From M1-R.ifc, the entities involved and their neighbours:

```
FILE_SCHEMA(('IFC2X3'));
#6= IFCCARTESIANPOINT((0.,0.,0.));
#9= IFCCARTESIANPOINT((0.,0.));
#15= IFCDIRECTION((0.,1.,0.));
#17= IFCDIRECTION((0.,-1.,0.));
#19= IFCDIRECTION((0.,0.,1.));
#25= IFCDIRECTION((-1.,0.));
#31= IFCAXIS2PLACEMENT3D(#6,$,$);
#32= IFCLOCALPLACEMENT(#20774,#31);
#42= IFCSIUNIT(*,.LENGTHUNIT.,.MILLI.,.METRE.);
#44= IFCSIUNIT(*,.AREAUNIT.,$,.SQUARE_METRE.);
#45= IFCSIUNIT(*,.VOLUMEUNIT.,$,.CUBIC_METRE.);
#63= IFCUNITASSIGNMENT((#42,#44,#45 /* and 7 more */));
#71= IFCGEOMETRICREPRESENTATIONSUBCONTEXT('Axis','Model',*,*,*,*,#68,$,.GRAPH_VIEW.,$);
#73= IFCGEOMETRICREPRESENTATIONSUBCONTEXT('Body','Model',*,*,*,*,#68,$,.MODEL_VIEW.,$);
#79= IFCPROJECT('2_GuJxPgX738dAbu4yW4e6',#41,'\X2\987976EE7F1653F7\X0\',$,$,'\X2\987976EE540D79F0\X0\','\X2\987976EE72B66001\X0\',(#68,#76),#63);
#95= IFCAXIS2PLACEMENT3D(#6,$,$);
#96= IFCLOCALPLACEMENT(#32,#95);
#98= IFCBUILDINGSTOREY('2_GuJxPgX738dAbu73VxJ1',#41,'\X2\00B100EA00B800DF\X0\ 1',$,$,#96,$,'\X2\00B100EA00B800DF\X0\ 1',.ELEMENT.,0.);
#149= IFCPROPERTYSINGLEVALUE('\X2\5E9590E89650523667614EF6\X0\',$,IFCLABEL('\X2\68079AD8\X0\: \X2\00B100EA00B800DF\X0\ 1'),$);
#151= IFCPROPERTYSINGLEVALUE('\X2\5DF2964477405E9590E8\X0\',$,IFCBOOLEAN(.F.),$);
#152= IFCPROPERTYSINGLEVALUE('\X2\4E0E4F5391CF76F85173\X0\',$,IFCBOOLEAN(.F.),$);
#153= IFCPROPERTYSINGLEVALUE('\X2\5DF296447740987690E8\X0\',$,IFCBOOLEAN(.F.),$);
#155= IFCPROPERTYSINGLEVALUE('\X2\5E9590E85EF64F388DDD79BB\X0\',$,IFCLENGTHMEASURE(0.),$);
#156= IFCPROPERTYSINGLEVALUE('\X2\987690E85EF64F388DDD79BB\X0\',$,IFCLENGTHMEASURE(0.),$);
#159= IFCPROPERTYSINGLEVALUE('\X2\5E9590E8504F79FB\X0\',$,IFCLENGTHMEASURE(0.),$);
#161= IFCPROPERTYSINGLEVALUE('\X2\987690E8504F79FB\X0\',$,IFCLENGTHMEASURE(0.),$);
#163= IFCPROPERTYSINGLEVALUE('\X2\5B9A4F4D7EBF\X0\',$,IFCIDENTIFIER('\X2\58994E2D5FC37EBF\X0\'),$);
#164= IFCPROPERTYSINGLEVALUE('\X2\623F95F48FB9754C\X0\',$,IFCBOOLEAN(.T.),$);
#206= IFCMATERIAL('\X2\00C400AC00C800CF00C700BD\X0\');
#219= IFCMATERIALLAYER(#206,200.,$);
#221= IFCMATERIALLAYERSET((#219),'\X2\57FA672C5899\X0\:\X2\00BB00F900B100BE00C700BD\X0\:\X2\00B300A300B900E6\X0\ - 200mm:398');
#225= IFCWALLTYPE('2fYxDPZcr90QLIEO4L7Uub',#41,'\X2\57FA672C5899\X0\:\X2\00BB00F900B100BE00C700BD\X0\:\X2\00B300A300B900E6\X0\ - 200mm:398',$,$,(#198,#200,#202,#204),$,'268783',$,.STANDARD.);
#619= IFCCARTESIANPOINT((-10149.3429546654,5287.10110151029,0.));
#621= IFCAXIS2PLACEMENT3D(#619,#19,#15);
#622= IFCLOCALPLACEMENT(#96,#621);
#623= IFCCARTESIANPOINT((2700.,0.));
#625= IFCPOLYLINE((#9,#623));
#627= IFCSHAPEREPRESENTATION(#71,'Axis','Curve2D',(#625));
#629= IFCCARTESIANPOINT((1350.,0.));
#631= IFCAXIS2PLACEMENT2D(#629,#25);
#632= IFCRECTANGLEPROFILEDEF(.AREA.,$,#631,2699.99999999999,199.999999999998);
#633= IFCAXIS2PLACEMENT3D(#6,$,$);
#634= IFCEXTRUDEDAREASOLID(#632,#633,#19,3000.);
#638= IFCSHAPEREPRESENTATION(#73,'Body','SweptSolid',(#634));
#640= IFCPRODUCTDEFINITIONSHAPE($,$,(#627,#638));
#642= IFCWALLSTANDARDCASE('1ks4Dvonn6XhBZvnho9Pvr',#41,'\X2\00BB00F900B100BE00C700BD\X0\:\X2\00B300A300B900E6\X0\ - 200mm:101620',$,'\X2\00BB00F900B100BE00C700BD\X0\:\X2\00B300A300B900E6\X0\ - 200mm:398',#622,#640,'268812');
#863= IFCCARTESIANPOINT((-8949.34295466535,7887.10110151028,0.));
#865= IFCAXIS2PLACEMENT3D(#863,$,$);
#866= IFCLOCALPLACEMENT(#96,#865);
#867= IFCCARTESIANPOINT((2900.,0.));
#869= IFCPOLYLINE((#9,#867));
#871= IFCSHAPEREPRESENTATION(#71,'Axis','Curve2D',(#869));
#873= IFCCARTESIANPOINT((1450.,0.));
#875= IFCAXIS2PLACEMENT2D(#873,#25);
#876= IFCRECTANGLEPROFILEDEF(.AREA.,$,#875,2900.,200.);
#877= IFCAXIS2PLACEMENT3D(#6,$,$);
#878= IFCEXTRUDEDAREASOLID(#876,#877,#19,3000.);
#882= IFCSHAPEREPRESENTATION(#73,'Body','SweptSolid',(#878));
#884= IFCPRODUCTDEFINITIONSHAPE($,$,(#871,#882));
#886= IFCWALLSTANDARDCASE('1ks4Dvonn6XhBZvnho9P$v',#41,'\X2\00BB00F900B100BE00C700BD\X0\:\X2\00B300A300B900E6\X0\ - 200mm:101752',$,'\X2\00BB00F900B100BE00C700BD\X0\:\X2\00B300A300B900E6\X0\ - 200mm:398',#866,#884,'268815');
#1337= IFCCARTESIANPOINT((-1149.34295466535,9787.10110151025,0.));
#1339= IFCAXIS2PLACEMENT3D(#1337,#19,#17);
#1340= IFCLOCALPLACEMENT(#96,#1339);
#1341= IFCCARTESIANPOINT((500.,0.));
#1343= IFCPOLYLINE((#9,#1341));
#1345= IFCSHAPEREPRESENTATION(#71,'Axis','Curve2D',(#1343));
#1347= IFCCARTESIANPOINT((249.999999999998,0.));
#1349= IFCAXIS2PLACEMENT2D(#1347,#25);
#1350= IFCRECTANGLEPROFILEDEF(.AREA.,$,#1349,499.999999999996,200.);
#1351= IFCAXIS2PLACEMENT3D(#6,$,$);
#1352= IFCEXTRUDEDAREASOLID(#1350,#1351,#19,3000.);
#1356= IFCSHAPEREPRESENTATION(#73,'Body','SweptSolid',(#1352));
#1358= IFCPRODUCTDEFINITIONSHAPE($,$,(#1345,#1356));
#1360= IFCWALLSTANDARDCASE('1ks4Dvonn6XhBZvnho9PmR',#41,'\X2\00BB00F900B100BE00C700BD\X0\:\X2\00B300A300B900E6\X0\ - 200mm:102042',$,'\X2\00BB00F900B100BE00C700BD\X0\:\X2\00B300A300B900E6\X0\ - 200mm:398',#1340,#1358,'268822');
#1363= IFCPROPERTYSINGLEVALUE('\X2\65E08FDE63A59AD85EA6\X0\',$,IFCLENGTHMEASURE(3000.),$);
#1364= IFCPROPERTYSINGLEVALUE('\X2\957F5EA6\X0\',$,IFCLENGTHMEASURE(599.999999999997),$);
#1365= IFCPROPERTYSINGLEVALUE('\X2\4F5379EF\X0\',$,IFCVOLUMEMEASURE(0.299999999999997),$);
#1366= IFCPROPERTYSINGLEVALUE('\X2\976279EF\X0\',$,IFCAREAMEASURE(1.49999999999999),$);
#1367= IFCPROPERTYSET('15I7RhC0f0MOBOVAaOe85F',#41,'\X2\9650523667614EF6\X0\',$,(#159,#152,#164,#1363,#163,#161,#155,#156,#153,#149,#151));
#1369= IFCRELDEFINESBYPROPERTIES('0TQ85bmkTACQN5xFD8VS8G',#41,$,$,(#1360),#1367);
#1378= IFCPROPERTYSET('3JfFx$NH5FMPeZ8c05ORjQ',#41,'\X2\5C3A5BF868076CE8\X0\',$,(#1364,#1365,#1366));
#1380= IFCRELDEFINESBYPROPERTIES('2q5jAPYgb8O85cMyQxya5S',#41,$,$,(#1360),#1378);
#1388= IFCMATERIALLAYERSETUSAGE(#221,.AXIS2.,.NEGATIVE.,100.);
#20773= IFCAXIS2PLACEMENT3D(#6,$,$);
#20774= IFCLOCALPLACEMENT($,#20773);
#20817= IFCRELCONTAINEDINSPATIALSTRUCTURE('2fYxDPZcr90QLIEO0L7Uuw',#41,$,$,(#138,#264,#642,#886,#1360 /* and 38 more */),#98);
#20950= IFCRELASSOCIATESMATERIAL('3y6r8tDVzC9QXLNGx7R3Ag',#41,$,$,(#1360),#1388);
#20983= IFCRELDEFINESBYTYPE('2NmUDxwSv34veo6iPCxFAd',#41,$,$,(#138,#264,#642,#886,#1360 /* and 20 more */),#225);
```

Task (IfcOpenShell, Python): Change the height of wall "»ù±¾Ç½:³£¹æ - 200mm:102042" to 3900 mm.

```python
import ifcopenshell
import ifcopenshell.api.pset
import ifcopenshell.geom
import ifcopenshell.util.element
import ifcopenshell.util.representation
import ifcopenshell.util.shape
import ifcopenshell.util.unit

model = ifcopenshell.open("M1-R.ifc")
area_scale = ifcopenshell.util.unit.calculate_unit_scale(model, "AREAUNIT")
volume_scale = ifcopenshell.util.unit.calculate_unit_scale(model, "VOLUMEUNIT")
settings = ifcopenshell.geom.settings()


def volume(element):
    """Net volume in cubic metres, openings subtracted."""
    shape = ifcopenshell.geom.create_shape(settings, element)
    return ifcopenshell.util.shape.get_volume(shape.geometry)


wall = model.by_id(1360)
before = volume(wall)

body = ifcopenshell.util.representation.get_representation(wall, "Model", "Body")
solid = body.Items[0]
old_height = solid.Depth
solid.Depth = 3900.0
after = volume(wall)
thickness = 0.2  # wall thickness in metres

# Update the stored height, areas and volumes.
pset = model.by_id(ifcopenshell.util.element.get_pset(wall, "限制条件", should_inherit=False)["id"])
ifcopenshell.api.pset.edit_pset(model, pset=pset, properties={
    "无连接高度": model.create_entity("IfcLengthMeasure", solid.Depth),
})
pset = model.by_id(ifcopenshell.util.element.get_pset(wall, "尺寸标注", should_inherit=False)["id"])
ifcopenshell.api.pset.edit_pset(model, pset=pset, properties={
    "体积": model.create_entity("IfcVolumeMeasure", after / volume_scale),
    "面积": model.create_entity("IfcAreaMeasure", after / thickness / area_scale),
})

print(f"height {old_height:g} -> {solid.Depth:g}, volume {before:.3f} -> {after:.3f} m3")

model.write("M1-R-out.ifc")
```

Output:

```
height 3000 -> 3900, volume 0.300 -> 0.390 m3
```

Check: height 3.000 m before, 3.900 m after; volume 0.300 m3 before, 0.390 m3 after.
